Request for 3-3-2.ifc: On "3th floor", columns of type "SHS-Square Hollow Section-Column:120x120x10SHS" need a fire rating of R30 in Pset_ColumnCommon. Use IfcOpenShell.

First a look at what the model holds.

```python
import ifcopenshell
import ifcopenshell.util.element

model = ifcopenshell.open("3-3-2.ifc")
print(model.schema)
storey = next(s for s in model.by_type("IfcBuildingStorey") if s.Name == "3th floor")
columns = [e for e in ifcopenshell.util.element.get_decomposition(storey) if e.is_a("IfcColumn")]
seen = {}
for e in columns:
    element_type = ifcopenshell.util.element.get_type(e)
    key = (element_type.Name if element_type != e and element_type else None, ifcopenshell.util.element.get_pset(e, "Pset_ColumnCommon", "FireRating"))
    seen[key] = seen.get(key, 0) + 1
for (name, value), count in sorted(seen.items(), key=str):
    print(count, "x", name, "|", value)
```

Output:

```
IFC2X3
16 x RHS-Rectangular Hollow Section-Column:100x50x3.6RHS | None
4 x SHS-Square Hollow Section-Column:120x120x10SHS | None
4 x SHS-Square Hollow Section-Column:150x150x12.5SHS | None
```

```python
import ifcopenshell
import ifcopenshell.api.pset
import ifcopenshell.util.element

model = ifcopenshell.open("3-3-2.ifc")

storey = next(s for s in model.by_type("IfcBuildingStorey") if s.Name == "3th floor")
columns = [e for e in ifcopenshell.util.element.get_decomposition(storey) if e.is_a("IfcColumn")]

count = 0
for e in columns:
    element_type = ifcopenshell.util.element.get_type(e)
    if element_type in (None, e) or element_type.Name != "SHS-Square Hollow Section-Column:120x120x10SHS":
        continue
    # add_pset returns the element's existing set when there is one.
    pset = ifcopenshell.api.pset.add_pset(model, product=e, name="Pset_ColumnCommon")
    ifcopenshell.api.pset.edit_pset(model, pset=pset, properties={"FireRating": "R30"})
    count += 1

print(count, "columns updated")

model.write("3-3-2-out.ifc")
```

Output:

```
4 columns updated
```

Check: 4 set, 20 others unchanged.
